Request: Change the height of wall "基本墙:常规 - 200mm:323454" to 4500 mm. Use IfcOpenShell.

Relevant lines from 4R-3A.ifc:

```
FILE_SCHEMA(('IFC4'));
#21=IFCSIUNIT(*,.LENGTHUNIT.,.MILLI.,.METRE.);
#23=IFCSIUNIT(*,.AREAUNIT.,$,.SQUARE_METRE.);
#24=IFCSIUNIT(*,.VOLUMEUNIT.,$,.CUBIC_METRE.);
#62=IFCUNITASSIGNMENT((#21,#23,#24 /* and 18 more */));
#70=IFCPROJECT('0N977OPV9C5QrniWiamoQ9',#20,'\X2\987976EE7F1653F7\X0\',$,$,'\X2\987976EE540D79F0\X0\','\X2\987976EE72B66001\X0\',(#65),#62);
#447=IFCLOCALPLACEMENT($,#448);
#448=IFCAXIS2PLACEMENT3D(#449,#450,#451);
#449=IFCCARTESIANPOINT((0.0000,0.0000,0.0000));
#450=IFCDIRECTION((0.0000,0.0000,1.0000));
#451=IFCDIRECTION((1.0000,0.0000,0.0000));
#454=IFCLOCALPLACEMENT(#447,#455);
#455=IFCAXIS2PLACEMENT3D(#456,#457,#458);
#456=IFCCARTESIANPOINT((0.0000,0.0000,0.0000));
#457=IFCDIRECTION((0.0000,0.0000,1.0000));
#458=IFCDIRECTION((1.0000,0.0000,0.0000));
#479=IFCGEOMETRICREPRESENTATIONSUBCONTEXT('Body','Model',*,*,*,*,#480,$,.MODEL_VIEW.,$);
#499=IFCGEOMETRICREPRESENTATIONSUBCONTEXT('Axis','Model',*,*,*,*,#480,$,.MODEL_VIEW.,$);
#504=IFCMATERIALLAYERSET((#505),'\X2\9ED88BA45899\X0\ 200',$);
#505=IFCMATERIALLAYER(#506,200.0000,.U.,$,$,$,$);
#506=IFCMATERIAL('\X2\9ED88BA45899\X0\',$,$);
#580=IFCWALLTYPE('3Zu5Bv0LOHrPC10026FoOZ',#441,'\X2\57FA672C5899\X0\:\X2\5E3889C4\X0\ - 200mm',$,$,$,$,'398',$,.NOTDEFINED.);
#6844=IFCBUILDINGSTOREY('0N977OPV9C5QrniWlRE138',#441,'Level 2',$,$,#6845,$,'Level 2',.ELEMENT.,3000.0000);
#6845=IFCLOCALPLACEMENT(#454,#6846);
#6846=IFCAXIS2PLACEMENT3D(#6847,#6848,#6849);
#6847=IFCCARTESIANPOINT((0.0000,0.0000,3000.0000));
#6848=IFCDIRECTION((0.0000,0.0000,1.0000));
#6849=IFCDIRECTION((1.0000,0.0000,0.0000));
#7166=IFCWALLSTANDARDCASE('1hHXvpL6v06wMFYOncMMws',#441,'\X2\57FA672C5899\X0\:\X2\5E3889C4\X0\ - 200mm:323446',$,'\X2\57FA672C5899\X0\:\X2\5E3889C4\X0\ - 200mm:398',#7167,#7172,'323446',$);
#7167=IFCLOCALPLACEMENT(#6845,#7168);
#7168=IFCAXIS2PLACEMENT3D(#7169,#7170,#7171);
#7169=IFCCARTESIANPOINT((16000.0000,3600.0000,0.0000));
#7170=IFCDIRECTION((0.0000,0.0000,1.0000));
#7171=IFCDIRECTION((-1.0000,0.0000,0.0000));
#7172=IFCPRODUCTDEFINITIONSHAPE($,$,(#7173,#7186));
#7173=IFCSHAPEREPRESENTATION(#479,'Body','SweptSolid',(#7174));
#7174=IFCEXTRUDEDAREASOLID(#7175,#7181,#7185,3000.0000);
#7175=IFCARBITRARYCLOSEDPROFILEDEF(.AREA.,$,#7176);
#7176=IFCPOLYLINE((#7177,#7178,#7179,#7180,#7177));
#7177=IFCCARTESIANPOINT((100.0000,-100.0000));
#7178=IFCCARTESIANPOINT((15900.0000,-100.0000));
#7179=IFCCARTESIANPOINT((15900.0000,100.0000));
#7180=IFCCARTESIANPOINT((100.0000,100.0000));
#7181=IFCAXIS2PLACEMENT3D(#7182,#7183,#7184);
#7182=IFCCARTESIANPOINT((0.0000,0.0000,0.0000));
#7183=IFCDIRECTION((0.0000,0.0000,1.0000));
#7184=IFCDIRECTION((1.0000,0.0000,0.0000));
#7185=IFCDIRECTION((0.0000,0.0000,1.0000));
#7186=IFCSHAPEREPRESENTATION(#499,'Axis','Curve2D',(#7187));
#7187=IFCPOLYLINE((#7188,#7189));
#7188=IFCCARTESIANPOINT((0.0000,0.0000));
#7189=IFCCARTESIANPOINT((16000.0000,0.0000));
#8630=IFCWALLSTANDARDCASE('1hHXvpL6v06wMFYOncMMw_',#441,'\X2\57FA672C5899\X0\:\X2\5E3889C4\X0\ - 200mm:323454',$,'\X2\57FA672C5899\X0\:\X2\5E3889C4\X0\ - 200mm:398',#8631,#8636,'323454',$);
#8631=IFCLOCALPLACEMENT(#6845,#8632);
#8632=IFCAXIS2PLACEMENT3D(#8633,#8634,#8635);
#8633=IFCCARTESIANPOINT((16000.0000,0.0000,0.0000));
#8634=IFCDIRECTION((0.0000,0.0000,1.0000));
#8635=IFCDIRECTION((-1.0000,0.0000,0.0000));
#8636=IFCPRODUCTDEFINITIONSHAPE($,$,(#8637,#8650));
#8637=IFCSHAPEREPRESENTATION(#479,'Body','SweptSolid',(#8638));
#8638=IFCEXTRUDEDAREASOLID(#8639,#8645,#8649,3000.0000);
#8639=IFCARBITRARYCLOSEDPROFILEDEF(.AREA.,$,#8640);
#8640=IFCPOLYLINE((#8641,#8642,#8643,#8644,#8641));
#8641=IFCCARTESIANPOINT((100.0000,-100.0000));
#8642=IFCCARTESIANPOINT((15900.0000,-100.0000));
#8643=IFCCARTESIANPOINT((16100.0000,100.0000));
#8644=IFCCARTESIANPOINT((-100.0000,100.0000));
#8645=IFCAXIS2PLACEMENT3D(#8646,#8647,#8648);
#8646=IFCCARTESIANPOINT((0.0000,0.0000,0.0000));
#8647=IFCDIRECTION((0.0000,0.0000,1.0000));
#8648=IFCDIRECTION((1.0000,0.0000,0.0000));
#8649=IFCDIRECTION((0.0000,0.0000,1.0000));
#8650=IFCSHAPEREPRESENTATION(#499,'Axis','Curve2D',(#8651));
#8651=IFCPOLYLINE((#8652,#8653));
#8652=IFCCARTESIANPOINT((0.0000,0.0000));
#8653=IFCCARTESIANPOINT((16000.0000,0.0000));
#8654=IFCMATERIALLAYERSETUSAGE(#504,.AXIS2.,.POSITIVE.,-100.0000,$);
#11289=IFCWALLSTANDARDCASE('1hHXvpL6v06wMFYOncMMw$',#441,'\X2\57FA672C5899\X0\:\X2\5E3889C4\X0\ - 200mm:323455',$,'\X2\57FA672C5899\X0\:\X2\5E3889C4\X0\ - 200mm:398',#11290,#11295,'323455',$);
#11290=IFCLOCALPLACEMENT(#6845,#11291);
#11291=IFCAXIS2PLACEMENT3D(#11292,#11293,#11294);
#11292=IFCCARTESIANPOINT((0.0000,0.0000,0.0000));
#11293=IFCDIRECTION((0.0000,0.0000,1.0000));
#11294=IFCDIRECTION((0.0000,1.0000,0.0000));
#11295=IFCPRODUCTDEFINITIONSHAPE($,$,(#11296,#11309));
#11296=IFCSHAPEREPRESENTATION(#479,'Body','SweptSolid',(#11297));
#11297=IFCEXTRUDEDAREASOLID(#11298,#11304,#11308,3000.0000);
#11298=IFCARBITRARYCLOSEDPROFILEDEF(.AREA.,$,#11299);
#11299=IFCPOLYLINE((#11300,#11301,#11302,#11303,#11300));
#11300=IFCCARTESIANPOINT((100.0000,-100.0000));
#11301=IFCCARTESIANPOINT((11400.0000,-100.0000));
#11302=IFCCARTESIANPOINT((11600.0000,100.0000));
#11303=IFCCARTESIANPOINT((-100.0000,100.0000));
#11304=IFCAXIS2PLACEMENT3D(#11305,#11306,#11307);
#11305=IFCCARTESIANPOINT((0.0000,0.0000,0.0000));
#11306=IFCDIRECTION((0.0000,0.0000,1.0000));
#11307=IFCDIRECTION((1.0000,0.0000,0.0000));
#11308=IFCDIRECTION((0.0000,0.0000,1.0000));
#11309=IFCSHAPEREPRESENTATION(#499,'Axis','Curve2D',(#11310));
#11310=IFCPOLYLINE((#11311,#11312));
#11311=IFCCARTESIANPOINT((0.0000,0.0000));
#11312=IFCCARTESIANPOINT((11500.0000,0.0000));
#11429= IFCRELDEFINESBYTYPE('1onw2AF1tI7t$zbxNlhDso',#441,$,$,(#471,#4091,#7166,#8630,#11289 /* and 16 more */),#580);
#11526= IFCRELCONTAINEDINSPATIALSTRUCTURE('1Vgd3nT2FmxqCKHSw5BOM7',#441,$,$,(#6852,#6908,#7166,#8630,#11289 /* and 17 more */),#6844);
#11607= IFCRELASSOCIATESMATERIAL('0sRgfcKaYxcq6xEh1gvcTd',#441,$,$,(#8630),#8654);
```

```python
import ifcopenshell
import ifcopenshell.geom
import ifcopenshell.util.representation
import ifcopenshell.util.shape

model = ifcopenshell.open("4R-3A.ifc")
settings = ifcopenshell.geom.settings()


def volume(element):
    """Net volume in cubic metres, openings subtracted."""
    shape = ifcopenshell.geom.create_shape(settings, element)
    return ifcopenshell.util.shape.get_volume(shape.geometry)


wall = model.by_guid("1hHXvpL6v06wMFYOncMMw_")
before = volume(wall)

body = ifcopenshell.util.representation.get_representation(wall, "Model", "Body")
solid = body.Items[0]
old_height = solid.Depth
solid.Depth = 4500.0
after = volume(wall)

print(f"height {old_height:g} -> {solid.Depth:g}, volume {before:.3f} -> {after:.3f} m3")

model.write("4R-3A_rev.ifc")
```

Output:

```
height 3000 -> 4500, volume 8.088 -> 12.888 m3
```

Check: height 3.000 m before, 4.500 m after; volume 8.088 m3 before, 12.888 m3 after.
